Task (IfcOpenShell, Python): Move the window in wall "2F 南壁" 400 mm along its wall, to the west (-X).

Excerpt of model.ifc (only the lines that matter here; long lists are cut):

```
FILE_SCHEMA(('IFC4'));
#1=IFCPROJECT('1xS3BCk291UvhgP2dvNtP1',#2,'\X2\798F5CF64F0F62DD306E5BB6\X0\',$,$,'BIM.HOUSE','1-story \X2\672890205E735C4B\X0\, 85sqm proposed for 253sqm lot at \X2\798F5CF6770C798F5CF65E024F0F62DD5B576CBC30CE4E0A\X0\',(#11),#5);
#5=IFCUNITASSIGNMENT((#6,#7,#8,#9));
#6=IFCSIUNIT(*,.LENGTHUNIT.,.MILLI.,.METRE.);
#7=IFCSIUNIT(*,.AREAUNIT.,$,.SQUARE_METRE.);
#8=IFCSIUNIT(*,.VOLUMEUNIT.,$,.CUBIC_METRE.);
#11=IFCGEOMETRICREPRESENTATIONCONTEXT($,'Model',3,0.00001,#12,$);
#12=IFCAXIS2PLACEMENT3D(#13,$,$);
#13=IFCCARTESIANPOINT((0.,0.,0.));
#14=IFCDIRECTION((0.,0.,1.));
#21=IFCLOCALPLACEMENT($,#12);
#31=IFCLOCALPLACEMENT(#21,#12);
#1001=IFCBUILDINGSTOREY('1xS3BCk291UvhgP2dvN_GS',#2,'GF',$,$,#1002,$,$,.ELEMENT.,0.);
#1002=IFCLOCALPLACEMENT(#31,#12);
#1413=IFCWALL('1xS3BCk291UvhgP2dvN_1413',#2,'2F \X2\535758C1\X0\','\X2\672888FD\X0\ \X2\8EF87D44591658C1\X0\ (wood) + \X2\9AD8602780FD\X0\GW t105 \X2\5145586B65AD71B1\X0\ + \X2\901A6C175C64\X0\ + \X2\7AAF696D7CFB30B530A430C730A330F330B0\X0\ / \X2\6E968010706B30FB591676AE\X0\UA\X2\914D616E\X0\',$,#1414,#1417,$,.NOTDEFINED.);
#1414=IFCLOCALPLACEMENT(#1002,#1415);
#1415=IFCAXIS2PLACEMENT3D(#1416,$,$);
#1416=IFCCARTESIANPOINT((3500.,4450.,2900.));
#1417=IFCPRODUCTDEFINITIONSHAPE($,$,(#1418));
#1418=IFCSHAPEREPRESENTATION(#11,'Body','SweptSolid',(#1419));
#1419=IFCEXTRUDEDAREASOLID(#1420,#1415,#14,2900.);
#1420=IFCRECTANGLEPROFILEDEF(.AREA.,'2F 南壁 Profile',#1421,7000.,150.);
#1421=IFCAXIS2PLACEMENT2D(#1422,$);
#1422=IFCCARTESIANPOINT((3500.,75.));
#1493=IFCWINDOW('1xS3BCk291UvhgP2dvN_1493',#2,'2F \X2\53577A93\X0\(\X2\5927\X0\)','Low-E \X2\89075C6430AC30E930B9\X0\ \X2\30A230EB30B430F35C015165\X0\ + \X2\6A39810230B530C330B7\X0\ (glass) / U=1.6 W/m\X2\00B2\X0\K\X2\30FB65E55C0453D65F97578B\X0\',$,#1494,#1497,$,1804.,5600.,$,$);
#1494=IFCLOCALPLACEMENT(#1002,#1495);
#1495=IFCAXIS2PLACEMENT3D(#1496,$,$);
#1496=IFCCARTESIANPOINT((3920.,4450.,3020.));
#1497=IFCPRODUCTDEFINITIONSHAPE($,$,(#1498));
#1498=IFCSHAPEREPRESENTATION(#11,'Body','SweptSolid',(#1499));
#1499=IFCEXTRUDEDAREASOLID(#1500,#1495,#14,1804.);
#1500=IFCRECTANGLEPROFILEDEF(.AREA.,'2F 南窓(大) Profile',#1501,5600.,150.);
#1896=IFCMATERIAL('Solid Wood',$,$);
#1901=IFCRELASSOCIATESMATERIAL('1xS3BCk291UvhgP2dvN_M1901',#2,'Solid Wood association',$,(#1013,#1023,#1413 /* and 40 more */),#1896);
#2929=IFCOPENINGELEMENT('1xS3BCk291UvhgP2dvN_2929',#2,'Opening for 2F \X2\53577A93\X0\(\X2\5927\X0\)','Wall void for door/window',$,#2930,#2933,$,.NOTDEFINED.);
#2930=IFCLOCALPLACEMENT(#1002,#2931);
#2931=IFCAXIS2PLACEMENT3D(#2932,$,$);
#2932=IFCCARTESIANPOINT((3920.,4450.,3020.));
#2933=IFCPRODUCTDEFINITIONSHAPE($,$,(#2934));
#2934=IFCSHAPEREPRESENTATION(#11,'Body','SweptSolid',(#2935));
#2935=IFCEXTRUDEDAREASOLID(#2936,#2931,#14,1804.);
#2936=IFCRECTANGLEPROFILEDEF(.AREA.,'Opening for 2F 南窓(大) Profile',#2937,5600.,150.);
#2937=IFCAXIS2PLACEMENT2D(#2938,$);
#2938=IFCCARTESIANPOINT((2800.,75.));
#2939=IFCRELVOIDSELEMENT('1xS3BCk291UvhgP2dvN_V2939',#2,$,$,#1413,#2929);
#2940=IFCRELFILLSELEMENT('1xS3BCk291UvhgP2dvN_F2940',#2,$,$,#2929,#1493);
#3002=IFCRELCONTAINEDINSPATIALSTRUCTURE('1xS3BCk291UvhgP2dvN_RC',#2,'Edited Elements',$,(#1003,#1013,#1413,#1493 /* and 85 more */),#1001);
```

```python
import ifcopenshell
import ifcopenshell.api.geometry
import ifcopenshell.util.placement
import ifcopenshell.util.unit

model = ifcopenshell.open("model.ifc")
unit_scale = ifcopenshell.util.unit.calculate_unit_scale(model)

window = model.by_id(1493)
opening = window.FillsVoids[0].RelatingOpeningElement
wall = opening.VoidsElements[0].RelatingBuildingElement

wall_matrix = ifcopenshell.util.placement.get_local_placement(wall.ObjectPlacement)
shift = wall_matrix[:3, 0] * -0.4 / unit_scale
before = ifcopenshell.util.placement.get_local_placement(window.ObjectPlacement)[:3, 3].copy()

# The window is not placed relative to its opening, so move both.
for product in (opening, window):
    matrix = ifcopenshell.util.placement.get_local_placement(product.ObjectPlacement)
    matrix[:3, 3] += shift
    ifcopenshell.api.geometry.edit_object_placement(model, product=product, matrix=matrix, is_si=False)

after = ifcopenshell.util.placement.get_local_placement(window.ObjectPlacement)[:3, 3]
print("window moved by", (after - before).round(3) + 0.0)

model.write("model_v2.ifc")
```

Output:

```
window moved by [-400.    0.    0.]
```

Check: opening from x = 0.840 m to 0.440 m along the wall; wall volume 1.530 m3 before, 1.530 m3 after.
